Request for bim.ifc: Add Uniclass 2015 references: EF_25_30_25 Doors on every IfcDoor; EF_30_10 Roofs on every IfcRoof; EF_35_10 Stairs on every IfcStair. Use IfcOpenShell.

First a look at what the model holds.

```python
import ifcopenshell

model = ifcopenshell.open("bim.ifc")
print(model.schema)
print("classifications:", [c.Name for c in model.by_type("IfcClassification")])
for ifc_class in ("IfcDoor", "IfcRoof", "IfcStair", "IfcWall", "IfcWindow"):
    print(ifc_class, len(model.by_type(ifc_class)))
```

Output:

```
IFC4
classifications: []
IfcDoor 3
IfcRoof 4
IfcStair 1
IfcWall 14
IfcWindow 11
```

```python
import ifcopenshell
import ifcopenshell.api.classification

model = ifcopenshell.open("bim.ifc")

system = ifcopenshell.api.classification.add_classification(model, classification="Uniclass 2015")

codes = {
    "IfcDoor": ("EF_25_30_25", "Doors"),
    "IfcRoof": ("EF_30_10", "Roofs"),
    "IfcStair": ("EF_35_10", "Stairs"),
}
for ifc_class, (code, name) in codes.items():
    products = model.by_type(ifc_class)
    ifcopenshell.api.classification.add_reference(
        model, products=products, classification=system, identification=code, name=name
    )
    print(code, len(products))

model.write("bim_updated.ifc")
```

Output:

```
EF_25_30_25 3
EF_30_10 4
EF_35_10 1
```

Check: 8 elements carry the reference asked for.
